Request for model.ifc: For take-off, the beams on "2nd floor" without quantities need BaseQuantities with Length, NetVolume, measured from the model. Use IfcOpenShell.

First a look at what the model holds.

```python
import ifcopenshell
import ifcopenshell.util.element
import ifcopenshell.util.unit

model = ifcopenshell.open("model.ifc")
print(model.schema)
for unit_type in ("LENGTHUNIT", "AREAUNIT", "VOLUMEUNIT"):
    print(unit_type, ifcopenshell.util.unit.calculate_unit_scale(model, unit_type))
storey = next(s for s in model.by_type("IfcBuildingStorey") if s.Name == "2nd floor")
beams = [e for e in ifcopenshell.util.element.get_decomposition(storey) if e.is_a("IfcBeam")]
for e in sorted(beams, key=lambda e: e.id()):
    print(e.id(), e.is_a(), e.Name, list(ifcopenshell.util.element.get_psets(e, qtos_only=True)), sep=" | ")
```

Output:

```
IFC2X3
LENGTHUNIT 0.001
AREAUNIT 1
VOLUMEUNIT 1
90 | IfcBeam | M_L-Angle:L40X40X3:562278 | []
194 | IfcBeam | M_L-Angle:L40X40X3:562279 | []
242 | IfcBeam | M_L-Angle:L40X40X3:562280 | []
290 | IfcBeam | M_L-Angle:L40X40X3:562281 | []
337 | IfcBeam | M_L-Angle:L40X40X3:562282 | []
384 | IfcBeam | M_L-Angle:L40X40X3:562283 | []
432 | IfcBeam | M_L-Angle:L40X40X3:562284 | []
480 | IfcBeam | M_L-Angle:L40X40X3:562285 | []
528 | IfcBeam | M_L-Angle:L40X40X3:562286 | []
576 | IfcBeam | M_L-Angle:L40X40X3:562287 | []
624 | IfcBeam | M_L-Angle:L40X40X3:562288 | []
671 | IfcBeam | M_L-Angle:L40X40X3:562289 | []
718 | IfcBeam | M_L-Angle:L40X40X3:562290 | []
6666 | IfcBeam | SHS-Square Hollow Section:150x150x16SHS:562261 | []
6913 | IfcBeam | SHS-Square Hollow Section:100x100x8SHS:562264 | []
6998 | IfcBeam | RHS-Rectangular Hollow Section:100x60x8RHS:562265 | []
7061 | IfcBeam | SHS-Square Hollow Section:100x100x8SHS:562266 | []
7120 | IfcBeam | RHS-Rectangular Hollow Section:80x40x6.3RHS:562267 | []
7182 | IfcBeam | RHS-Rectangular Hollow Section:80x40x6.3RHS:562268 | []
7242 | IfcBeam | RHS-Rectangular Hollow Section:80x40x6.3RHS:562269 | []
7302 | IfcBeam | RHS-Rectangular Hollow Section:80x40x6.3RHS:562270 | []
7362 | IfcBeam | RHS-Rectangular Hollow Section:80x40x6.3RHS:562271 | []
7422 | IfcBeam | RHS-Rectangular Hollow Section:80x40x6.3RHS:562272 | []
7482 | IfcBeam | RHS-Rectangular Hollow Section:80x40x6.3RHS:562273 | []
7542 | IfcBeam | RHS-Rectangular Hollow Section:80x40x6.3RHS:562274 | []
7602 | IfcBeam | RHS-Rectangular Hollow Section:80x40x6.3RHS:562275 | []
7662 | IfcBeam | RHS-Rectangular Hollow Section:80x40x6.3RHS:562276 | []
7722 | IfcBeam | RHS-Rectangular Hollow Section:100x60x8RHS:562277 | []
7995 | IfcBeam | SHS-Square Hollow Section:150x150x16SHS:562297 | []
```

```python
import ifcopenshell
import ifcopenshell.api.pset
import ifcopenshell.geom
import ifcopenshell.util.element
import ifcopenshell.util.shape
import ifcopenshell.util.unit

model = ifcopenshell.open("model.ifc")
unit_scale = ifcopenshell.util.unit.calculate_unit_scale(model)
volume_scale = ifcopenshell.util.unit.calculate_unit_scale(model, "VOLUMEUNIT")
settings = ifcopenshell.geom.settings()

storey = next(s for s in model.by_type("IfcBuildingStorey") if s.Name == "2nd floor")
beams = [e for e in ifcopenshell.util.element.get_decomposition(storey) if e.is_a("IfcBeam")]

for e in sorted(beams, key=lambda e: e.id()):
    if ifcopenshell.util.element.get_psets(e, qtos_only=True, should_inherit=False):
        continue
    # Geometry comes back in metres, in the element's own axes.
    shape = ifcopenshell.geom.create_shape(settings, e)
    values = {
        "Length": ifcopenshell.util.shape.get_max_xyz(shape.geometry) / unit_scale,
        "NetVolume": ifcopenshell.util.shape.get_volume(shape.geometry) / volume_scale,
    }
    qto = ifcopenshell.api.pset.add_qto(model, product=e, name="BaseQuantities")
    ifcopenshell.api.pset.edit_qto(model, qto=qto, properties=values)
    print(e.id(), {k: round(v, 3) for k, v in values.items()})

model.write("model_edited.ifc")
```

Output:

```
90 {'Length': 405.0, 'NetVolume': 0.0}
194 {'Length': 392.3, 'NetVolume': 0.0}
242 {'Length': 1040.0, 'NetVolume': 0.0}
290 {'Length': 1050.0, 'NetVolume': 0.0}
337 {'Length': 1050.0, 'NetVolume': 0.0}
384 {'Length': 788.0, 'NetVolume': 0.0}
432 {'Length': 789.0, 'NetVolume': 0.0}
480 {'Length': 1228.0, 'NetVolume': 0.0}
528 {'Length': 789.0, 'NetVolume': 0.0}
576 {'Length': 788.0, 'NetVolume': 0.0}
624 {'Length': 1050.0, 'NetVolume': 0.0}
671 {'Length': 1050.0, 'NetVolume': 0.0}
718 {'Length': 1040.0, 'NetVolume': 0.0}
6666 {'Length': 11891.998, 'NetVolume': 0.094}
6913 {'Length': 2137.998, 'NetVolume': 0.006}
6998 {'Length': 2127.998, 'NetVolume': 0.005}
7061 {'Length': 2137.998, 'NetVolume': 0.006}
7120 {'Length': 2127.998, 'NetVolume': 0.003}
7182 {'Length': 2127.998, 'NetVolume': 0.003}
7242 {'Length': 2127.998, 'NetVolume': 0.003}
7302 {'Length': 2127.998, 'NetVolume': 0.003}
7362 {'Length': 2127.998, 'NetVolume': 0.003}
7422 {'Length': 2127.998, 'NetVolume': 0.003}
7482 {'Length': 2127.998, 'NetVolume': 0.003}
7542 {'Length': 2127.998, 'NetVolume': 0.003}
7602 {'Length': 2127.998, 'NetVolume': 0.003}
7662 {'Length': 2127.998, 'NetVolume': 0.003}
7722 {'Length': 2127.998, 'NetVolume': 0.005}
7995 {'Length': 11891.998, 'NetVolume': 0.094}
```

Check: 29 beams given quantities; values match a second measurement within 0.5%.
